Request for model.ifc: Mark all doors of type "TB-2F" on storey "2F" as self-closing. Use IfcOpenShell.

First a look at what the model holds.

```python
import ifcopenshell
import ifcopenshell.util.element

model = ifcopenshell.open("model.ifc")
print(model.schema)
storey = next(s for s in model.by_type("IfcBuildingStorey") if s.Name == "2F")
doors = [e for e in ifcopenshell.util.element.get_decomposition(storey) if e.is_a("IfcDoor")]
seen = {}
for e in doors:
    element_type = ifcopenshell.util.element.get_type(e)
    key = (element_type.Name if element_type != e and element_type else None, ifcopenshell.util.element.get_pset(e, "Pset_DoorCommon", "SelfClosing"))
    seen[key] = seen.get(key, 0) + 1
for (name, value), count in sorted(seen.items(), key=str):
    print(count, "x", name, "|", value)
```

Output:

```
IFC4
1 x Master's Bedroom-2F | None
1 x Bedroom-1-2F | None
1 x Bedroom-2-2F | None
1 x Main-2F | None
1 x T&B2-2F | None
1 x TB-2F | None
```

```python
import ifcopenshell
import ifcopenshell.api.pset
import ifcopenshell.util.element

model = ifcopenshell.open("model.ifc")

storey = next(s for s in model.by_type("IfcBuildingStorey") if s.Name == "2F")
doors = [e for e in ifcopenshell.util.element.get_decomposition(storey) if e.is_a("IfcDoor")]

count = 0
for e in doors:
    element_type = ifcopenshell.util.element.get_type(e)
    if element_type in (None, e) or element_type.Name != "TB-2F":
        continue
    # add_pset returns the element's existing set when there is one.
    pset = ifcopenshell.api.pset.add_pset(model, product=e, name="Pset_DoorCommon")
    ifcopenshell.api.pset.edit_pset(model, pset=pset, properties={"SelfClosing": True})
    count += 1

print(count, "doors updated")

model.write("model-out.ifc")
```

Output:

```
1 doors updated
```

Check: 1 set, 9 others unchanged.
